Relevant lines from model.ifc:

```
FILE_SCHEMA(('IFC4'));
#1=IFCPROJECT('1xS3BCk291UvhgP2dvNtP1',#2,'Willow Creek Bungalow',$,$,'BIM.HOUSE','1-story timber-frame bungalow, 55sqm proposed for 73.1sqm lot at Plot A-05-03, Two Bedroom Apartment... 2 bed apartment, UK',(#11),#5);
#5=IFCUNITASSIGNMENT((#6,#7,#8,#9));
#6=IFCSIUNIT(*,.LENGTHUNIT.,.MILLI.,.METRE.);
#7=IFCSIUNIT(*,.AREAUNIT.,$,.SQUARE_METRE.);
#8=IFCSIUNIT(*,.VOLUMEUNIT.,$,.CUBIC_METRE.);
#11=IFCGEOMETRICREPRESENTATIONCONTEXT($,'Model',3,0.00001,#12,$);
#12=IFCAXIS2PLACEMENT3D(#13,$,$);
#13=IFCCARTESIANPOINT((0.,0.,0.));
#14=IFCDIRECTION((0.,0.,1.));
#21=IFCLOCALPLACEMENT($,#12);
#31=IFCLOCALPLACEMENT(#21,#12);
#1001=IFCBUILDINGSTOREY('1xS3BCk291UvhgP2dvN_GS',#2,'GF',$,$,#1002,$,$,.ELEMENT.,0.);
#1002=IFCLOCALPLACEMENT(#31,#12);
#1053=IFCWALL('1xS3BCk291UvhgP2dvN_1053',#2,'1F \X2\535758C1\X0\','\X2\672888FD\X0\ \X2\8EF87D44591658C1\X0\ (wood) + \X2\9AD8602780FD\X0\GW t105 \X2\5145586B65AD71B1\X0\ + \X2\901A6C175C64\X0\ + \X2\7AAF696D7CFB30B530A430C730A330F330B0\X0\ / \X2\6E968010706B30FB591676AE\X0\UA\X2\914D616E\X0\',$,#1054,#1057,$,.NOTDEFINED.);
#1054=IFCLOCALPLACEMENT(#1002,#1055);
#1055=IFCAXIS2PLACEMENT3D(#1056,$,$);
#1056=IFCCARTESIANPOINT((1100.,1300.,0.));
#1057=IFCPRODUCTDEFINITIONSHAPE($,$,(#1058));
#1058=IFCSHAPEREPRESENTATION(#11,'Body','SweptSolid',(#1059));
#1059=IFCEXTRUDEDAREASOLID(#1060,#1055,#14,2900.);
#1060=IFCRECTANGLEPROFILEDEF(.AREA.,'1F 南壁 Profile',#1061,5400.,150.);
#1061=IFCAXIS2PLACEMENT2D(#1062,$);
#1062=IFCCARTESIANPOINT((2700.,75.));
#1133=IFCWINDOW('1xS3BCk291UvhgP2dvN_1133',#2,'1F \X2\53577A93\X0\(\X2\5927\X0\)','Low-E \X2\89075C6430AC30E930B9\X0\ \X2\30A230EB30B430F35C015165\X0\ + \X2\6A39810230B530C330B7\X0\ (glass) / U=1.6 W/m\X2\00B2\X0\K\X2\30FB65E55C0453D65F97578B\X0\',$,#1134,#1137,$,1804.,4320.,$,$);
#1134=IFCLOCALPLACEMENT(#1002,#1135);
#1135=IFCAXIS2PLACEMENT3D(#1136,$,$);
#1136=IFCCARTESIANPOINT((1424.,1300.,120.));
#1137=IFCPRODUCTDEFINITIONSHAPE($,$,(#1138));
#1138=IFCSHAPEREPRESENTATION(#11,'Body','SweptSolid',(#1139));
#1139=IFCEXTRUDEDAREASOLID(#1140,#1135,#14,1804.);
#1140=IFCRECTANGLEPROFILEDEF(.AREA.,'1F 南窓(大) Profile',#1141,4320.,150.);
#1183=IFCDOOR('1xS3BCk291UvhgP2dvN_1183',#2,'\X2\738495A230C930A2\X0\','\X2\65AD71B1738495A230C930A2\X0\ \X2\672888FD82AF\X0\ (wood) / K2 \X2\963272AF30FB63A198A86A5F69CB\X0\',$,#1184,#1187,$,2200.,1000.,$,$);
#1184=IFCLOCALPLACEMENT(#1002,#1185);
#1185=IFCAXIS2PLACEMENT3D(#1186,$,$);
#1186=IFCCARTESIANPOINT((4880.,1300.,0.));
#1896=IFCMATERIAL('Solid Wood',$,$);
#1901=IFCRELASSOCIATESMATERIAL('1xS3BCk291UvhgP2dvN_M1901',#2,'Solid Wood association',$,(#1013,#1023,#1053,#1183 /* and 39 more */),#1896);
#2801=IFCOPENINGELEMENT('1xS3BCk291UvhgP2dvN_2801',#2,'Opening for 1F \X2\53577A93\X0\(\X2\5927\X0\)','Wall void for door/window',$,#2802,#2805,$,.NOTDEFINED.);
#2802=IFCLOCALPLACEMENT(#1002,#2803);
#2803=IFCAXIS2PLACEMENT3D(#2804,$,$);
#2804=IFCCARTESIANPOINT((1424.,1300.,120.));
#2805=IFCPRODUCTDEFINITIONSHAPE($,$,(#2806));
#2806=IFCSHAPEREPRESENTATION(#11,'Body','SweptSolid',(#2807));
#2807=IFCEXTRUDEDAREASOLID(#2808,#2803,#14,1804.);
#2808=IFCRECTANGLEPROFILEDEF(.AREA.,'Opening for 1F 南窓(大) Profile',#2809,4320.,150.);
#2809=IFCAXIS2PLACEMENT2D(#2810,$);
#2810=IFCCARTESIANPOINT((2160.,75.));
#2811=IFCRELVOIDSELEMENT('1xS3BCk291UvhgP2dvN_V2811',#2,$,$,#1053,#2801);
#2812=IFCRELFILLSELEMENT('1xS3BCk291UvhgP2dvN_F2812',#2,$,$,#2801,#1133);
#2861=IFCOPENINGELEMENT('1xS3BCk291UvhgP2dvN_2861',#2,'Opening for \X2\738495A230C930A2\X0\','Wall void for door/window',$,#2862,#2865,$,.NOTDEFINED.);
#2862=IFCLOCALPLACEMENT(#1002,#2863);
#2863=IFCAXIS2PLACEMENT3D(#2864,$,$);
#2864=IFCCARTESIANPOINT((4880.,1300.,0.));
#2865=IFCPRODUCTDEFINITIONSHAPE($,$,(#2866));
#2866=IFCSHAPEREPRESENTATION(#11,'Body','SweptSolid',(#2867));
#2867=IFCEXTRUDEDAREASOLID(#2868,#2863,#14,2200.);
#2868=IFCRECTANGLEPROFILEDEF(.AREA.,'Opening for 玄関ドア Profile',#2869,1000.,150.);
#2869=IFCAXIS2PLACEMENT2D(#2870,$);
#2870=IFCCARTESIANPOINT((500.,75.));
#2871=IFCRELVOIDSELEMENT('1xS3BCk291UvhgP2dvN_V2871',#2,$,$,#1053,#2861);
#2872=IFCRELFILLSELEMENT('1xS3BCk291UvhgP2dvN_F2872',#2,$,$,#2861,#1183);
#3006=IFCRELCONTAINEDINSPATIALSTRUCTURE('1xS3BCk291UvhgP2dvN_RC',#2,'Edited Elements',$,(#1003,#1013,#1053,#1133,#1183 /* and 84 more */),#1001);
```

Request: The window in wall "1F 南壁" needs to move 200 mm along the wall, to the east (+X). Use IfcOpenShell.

```python
import ifcopenshell
import ifcopenshell.api.geometry
import ifcopenshell.util.placement
import ifcopenshell.util.unit

model = ifcopenshell.open("model.ifc")
unit_scale = ifcopenshell.util.unit.calculate_unit_scale(model)

window = model.by_guid("1xS3BCk291UvhgP2dvN_1133")
opening = window.FillsVoids[0].RelatingOpeningElement
wall = opening.VoidsElements[0].RelatingBuildingElement

wall_matrix = ifcopenshell.util.placement.get_local_placement(wall.ObjectPlacement)
shift = wall_matrix[:3, 0] * 0.2 / unit_scale
before = ifcopenshell.util.placement.get_local_placement(window.ObjectPlacement)[:3, 3].copy()

# The window is not placed relative to its opening, so move both.
for product in (opening, window):
    matrix = ifcopenshell.util.placement.get_local_placement(product.ObjectPlacement)
    matrix[:3, 3] += shift
    ifcopenshell.api.geometry.edit_object_placement(model, product=product, matrix=matrix, is_si=False)

after = ifcopenshell.util.placement.get_local_placement(window.ObjectPlacement)[:3, 3]
print("window moved by", (after - before).round(3) + 0.0)

model.write("model_rev.ifc")
```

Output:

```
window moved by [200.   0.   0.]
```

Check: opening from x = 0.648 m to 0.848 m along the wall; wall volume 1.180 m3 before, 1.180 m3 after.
